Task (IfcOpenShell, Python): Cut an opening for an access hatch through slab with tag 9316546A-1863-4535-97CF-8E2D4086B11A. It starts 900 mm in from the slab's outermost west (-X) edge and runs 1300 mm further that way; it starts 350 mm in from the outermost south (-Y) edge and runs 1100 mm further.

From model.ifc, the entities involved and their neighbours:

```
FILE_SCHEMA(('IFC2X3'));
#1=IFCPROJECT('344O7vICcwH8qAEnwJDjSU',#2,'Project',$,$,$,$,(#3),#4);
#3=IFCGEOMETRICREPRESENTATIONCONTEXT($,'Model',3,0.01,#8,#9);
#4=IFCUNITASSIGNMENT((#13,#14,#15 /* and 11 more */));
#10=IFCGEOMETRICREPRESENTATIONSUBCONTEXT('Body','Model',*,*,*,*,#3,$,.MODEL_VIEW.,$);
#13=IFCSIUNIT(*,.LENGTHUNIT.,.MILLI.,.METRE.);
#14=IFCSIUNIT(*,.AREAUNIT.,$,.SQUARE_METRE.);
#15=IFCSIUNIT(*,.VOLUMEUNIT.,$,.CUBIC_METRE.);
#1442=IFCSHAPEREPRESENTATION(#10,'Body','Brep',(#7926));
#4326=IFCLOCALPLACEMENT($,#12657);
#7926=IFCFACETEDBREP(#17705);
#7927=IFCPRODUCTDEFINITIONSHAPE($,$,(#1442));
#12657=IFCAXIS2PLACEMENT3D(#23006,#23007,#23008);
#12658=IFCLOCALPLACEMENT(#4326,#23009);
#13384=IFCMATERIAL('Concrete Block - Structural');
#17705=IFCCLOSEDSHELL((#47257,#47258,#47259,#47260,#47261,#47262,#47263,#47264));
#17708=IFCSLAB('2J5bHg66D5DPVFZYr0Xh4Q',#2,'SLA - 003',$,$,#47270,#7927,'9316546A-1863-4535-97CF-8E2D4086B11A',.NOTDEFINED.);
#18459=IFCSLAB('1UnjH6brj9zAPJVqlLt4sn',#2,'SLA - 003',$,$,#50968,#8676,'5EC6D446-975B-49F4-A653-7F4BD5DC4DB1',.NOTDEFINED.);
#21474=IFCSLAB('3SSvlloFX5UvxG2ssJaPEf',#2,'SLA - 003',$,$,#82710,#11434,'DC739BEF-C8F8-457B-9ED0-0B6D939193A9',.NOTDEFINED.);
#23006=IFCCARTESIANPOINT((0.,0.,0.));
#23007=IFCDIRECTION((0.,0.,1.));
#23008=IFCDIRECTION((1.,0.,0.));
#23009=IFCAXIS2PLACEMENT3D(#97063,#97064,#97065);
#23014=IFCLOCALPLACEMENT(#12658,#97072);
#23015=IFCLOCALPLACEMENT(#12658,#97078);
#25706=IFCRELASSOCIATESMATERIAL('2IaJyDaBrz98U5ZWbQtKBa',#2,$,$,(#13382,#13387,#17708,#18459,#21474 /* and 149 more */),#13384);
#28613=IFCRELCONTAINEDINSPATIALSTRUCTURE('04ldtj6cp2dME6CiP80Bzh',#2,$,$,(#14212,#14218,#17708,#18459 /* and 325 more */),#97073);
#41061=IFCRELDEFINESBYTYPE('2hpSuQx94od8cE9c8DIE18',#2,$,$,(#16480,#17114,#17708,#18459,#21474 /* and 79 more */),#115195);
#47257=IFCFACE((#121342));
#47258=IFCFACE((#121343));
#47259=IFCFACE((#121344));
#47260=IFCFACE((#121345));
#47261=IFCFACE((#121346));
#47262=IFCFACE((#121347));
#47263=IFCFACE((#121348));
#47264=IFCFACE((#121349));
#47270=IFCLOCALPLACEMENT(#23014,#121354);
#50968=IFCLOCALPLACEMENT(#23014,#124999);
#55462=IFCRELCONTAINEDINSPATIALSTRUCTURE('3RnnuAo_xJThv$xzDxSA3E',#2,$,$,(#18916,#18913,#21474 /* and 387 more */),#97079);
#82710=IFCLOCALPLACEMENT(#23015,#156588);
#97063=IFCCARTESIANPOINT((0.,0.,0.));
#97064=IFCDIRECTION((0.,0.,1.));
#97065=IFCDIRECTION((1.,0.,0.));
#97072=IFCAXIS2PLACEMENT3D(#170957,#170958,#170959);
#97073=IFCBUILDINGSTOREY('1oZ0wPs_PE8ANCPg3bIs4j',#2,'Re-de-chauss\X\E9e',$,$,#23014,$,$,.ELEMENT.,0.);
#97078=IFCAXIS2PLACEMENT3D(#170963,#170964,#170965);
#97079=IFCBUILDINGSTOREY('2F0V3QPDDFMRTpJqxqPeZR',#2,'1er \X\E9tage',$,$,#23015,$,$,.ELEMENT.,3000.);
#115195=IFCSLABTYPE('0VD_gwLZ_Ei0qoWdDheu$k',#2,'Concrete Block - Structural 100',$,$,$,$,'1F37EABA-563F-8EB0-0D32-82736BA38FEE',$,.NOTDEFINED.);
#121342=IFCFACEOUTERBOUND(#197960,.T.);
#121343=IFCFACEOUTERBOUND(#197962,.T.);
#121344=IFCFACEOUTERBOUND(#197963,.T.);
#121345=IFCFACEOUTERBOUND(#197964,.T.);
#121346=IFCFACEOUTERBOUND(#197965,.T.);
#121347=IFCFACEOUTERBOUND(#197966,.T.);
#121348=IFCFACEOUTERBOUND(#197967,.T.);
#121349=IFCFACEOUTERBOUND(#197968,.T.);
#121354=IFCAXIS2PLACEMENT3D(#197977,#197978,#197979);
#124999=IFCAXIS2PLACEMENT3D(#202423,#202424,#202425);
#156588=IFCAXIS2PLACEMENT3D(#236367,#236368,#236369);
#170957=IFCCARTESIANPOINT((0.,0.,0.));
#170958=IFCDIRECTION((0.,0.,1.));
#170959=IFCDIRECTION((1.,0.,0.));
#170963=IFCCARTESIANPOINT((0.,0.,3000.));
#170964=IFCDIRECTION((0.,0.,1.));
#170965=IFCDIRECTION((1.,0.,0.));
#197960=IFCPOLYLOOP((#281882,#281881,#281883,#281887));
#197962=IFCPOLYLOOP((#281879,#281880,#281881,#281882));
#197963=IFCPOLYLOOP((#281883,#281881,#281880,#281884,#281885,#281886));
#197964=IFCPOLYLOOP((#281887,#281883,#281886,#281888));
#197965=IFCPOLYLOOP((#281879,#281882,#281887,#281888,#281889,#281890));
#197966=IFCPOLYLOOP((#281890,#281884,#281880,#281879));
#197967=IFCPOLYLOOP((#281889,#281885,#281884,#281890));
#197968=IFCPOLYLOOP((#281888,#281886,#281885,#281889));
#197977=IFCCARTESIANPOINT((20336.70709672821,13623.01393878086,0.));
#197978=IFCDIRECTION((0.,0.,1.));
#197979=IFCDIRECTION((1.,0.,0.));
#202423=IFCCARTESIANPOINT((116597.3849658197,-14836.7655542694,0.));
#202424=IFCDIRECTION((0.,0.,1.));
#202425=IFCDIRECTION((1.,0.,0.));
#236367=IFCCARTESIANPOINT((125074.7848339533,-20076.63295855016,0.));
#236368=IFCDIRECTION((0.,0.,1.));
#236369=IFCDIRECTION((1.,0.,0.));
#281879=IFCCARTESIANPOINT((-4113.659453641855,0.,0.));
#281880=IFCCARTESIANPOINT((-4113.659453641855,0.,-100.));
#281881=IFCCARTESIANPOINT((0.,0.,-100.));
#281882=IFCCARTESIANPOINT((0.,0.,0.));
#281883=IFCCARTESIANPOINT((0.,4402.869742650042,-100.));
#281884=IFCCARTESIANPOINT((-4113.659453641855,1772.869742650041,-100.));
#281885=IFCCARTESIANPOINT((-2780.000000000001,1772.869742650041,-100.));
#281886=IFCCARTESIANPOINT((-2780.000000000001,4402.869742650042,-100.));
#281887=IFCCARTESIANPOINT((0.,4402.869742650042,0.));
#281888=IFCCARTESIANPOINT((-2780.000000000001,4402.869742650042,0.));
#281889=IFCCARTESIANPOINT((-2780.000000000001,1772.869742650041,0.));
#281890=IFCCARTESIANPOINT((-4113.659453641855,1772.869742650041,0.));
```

```python
import numpy as np
import ifcopenshell
import ifcopenshell.api.feature
import ifcopenshell.api.geometry
import ifcopenshell.api.root
import ifcopenshell.geom
import ifcopenshell.util.placement
import ifcopenshell.util.representation
import ifcopenshell.util.shape
import ifcopenshell.util.unit

model = ifcopenshell.open("model.ifc")
unit_scale = ifcopenshell.util.unit.calculate_unit_scale(model)
settings = ifcopenshell.geom.settings()


def volume(element):
    """Net volume in cubic metres, openings subtracted."""
    shape = ifcopenshell.geom.create_shape(settings, element)
    return ifcopenshell.util.shape.get_volume(shape.geometry)


slab = model.by_id(17708)
before = volume(slab)

# Extent in the slab's own axes, in metres. The edges named are its -X and -Y sides.
slab_shape = ifcopenshell.geom.create_shape(settings, slab)
vertices = ifcopenshell.util.shape.get_vertices(slab_shape.geometry)
x_min, y_min, bottom = vertices.min(axis=0)
top = vertices[:, 2].max()

opening = ifcopenshell.api.root.create_entity(model, ifc_class="IfcOpeningElement", name="Access hatch opening")
context = ifcopenshell.util.representation.get_context(model, "Model", "Body", "MODEL_VIEW")
width, depth = 1.3, 1.1
outline = [(0.0, 0.0), (width, 0.0), (width, depth), (0.0, depth), (0.0, 0.0)]
# Overshoot both faces by 50 mm so the cut is clean.
shape = ifcopenshell.api.geometry.add_slab_representation(
    model, context=context, depth=top - bottom + 0.1, polyline=outline
)
ifcopenshell.api.geometry.assign_representation(model, product=opening, representation=shape)

matrix = ifcopenshell.util.placement.get_local_placement(slab.ObjectPlacement)
matrix[:, 3] = matrix @ np.append(np.array([x_min + 0.9, y_min + 0.35, bottom - 0.05]) / unit_scale, 1.0)
ifcopenshell.api.geometry.edit_object_placement(model, product=opening, matrix=matrix, is_si=False)
ifcopenshell.api.feature.add_feature(model, feature=opening, element=slab)

after = volume(slab)

print(f"slab volume {before:.3f} -> {after:.3f} m3")

model.write("model_updated.ifc")
```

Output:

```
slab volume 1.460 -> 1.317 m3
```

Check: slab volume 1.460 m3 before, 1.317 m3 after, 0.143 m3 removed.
